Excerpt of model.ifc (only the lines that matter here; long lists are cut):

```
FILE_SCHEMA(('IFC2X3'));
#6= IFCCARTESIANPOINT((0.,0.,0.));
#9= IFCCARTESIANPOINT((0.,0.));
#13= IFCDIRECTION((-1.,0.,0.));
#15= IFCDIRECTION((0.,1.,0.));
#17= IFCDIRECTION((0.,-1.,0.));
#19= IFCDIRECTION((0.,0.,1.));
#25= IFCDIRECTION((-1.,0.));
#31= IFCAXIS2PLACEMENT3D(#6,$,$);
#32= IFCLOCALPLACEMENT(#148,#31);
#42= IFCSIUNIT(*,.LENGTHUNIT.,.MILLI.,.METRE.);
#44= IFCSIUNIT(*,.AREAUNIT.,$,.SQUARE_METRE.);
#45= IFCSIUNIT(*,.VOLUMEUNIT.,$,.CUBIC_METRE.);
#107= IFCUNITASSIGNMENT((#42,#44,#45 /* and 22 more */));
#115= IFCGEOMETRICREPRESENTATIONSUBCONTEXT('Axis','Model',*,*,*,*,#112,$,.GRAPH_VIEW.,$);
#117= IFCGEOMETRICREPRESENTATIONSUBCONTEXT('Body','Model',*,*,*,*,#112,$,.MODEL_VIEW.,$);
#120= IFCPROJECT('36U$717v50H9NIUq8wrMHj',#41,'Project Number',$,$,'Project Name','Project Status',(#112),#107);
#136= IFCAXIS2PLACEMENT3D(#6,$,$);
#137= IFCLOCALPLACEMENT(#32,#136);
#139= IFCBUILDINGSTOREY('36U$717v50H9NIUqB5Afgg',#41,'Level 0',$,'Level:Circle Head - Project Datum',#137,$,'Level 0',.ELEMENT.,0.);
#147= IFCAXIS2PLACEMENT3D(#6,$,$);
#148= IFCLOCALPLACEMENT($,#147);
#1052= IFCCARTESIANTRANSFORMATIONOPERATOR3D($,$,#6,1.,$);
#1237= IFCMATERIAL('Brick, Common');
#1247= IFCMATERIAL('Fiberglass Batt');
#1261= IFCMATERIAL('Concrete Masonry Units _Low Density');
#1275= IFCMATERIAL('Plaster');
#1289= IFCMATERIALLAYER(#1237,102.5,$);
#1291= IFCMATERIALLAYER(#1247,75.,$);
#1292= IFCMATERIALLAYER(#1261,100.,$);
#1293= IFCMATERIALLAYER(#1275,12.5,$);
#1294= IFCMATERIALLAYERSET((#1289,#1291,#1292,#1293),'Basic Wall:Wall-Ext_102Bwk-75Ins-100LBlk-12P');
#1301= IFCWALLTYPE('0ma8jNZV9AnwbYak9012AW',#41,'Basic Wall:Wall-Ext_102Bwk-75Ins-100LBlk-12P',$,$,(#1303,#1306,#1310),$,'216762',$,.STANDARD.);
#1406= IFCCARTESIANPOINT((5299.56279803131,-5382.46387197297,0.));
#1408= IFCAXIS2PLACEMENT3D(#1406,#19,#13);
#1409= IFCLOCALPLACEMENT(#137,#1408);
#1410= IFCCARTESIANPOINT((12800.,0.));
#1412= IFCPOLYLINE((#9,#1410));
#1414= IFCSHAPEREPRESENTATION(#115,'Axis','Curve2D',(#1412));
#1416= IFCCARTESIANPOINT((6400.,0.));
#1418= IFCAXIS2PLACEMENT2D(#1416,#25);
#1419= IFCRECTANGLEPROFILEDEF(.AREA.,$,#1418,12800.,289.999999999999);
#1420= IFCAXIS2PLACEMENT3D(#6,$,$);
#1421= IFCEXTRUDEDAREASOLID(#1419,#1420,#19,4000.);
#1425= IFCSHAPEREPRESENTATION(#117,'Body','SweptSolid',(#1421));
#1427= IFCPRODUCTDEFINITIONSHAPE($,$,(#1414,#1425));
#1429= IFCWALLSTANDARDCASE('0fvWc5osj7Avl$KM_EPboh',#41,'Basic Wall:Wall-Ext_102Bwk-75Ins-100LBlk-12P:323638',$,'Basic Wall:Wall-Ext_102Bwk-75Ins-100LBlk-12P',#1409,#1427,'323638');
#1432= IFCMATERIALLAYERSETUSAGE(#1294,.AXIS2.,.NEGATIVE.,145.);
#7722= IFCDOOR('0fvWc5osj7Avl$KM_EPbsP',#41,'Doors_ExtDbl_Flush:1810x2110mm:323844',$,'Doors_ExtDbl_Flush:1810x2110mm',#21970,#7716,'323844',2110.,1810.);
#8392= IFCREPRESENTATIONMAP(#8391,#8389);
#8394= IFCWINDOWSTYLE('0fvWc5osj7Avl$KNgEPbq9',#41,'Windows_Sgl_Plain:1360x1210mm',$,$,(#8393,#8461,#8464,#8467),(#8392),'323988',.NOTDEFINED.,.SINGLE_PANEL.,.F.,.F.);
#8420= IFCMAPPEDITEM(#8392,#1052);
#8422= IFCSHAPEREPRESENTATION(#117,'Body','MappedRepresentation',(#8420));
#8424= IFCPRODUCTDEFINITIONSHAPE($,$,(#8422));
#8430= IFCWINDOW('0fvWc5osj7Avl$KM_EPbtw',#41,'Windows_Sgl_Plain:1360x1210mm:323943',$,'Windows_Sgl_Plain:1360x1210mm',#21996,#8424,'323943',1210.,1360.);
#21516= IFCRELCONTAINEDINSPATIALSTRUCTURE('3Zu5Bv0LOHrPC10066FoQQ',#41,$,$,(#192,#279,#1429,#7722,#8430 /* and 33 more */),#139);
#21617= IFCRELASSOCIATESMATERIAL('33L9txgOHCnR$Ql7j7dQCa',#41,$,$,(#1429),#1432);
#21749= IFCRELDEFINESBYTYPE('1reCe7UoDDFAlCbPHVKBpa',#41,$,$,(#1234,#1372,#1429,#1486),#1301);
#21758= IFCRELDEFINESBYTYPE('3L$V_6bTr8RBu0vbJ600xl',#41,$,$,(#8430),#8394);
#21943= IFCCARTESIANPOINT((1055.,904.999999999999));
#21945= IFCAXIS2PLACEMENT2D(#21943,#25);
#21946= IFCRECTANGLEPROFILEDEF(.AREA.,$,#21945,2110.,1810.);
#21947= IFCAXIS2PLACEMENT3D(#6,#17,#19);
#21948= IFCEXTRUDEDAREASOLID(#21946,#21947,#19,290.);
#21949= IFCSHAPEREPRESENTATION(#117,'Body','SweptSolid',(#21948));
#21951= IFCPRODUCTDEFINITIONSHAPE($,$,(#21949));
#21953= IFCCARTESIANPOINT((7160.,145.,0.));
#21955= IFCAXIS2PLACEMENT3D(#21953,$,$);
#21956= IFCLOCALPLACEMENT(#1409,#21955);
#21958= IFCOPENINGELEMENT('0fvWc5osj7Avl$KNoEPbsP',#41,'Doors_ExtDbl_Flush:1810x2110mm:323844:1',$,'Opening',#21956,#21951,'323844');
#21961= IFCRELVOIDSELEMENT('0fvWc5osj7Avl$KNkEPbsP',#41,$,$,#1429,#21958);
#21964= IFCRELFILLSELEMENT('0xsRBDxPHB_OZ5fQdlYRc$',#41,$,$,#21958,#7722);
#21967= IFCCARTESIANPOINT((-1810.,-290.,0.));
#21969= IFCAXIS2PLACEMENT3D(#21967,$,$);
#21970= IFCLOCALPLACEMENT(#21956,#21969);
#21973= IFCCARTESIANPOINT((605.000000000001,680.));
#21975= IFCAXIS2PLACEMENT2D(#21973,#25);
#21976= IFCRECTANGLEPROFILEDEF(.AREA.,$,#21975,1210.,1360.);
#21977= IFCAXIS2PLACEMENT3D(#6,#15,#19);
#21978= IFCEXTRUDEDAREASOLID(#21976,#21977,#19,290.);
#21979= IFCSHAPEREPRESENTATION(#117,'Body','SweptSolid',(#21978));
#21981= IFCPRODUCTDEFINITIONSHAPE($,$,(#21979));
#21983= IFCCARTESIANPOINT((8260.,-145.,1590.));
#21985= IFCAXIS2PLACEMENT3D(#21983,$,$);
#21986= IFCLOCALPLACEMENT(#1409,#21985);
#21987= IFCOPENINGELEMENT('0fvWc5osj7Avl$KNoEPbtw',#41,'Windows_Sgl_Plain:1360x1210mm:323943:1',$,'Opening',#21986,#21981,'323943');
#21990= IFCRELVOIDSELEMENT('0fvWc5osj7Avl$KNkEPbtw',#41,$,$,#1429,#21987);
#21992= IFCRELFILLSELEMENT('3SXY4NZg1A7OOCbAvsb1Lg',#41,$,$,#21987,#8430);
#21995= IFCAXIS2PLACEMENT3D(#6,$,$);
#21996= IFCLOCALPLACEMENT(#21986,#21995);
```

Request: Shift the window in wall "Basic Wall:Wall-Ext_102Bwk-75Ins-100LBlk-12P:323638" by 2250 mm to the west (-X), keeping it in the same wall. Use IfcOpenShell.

```python
import ifcopenshell
import ifcopenshell.api.geometry
import ifcopenshell.util.placement
import ifcopenshell.util.unit

model = ifcopenshell.open("model.ifc")
unit_scale = ifcopenshell.util.unit.calculate_unit_scale(model)

window = model.by_id(8430)
opening = window.FillsVoids[0].RelatingOpeningElement
wall = opening.VoidsElements[0].RelatingBuildingElement

wall_matrix = ifcopenshell.util.placement.get_local_placement(wall.ObjectPlacement)
shift = wall_matrix[:3, 0] * 2.25 / unit_scale
before = ifcopenshell.util.placement.get_local_placement(window.ObjectPlacement)[:3, 3].copy()

# The window is placed relative to its opening, so it follows when the opening moves.
matrix = ifcopenshell.util.placement.get_local_placement(opening.ObjectPlacement)
matrix[:3, 3] += shift
ifcopenshell.api.geometry.edit_object_placement(
    model, product=opening, matrix=matrix, is_si=False, should_transform_children=True
)

after = ifcopenshell.util.placement.get_local_placement(window.ObjectPlacement)[:3, 3]
print("window moved by", (after - before).round(3) + 0.0)

model.write("model_v2.ifc")
```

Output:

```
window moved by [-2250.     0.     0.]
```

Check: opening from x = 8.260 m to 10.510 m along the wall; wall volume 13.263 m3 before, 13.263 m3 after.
